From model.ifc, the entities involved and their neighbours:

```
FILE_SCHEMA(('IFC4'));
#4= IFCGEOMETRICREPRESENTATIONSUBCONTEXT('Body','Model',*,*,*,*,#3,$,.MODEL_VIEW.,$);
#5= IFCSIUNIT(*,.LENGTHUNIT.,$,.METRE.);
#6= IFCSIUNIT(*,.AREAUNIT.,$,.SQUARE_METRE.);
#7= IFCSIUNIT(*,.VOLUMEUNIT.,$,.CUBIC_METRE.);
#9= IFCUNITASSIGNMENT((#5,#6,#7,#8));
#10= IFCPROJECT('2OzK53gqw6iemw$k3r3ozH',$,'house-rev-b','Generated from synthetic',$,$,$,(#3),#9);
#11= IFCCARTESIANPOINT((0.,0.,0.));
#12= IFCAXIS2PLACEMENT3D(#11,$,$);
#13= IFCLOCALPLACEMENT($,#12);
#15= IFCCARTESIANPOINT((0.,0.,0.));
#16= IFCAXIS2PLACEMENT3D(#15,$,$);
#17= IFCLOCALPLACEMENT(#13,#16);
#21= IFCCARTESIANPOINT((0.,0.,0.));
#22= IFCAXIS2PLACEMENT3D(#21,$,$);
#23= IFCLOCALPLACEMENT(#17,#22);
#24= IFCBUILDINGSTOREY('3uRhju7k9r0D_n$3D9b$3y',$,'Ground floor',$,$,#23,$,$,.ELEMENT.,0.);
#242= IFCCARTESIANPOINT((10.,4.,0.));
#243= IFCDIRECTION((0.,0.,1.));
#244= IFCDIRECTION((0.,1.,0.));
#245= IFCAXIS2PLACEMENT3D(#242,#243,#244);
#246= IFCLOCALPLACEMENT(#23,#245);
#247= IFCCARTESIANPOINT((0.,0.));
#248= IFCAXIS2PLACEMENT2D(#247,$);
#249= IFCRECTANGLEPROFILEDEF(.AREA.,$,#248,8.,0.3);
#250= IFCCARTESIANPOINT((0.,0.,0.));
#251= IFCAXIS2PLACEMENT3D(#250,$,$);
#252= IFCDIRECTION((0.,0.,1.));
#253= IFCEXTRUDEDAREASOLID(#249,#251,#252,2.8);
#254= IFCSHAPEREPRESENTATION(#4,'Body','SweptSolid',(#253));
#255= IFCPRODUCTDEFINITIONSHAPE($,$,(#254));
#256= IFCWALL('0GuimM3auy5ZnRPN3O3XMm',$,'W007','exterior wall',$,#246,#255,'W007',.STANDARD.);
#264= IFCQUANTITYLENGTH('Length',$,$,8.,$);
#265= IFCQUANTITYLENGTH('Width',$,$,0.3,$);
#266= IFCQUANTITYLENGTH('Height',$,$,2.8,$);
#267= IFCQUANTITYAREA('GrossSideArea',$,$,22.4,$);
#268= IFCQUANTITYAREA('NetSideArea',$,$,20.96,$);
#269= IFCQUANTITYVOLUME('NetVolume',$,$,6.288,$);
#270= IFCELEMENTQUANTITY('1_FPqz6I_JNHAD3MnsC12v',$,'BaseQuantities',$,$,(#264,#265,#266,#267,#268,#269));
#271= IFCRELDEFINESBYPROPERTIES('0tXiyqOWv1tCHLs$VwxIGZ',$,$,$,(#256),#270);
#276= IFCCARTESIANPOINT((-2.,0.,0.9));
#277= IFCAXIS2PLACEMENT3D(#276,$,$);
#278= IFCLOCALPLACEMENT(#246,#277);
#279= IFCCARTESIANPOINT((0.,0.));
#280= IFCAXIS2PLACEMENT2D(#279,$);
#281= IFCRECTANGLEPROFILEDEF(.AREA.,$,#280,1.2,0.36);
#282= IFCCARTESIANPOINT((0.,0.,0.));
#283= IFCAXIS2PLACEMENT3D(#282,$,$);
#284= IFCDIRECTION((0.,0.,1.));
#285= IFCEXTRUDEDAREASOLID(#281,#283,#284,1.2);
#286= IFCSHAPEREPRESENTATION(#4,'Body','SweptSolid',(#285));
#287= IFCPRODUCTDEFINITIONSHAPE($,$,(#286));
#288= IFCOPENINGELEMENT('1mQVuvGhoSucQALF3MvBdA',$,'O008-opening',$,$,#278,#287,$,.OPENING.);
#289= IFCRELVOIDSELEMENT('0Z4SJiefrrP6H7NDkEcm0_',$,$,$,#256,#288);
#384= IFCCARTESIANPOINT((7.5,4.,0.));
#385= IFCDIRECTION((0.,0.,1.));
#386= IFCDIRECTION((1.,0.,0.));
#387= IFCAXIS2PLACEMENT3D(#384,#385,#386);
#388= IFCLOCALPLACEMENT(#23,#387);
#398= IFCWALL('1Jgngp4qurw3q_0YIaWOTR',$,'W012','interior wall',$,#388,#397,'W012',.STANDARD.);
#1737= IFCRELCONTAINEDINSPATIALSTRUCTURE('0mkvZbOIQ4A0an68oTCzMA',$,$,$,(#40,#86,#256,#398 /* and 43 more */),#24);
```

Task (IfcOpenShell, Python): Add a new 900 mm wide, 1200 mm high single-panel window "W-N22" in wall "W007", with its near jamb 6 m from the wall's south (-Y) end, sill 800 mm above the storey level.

```python
import numpy as np
import ifcopenshell
import ifcopenshell.api.feature
import ifcopenshell.api.geometry
import ifcopenshell.api.pset
import ifcopenshell.api.root
import ifcopenshell.api.spatial
import ifcopenshell.geom
import ifcopenshell.util.element
import ifcopenshell.util.placement
import ifcopenshell.util.representation
import ifcopenshell.util.shape
import ifcopenshell.util.unit

model = ifcopenshell.open("model.ifc")
unit_scale = ifcopenshell.util.unit.calculate_unit_scale(model)
area_scale = ifcopenshell.util.unit.calculate_unit_scale(model, "AREAUNIT")
volume_scale = ifcopenshell.util.unit.calculate_unit_scale(model, "VOLUMEUNIT")
settings = ifcopenshell.geom.settings()


def volume(element):
    """Net volume in cubic metres, openings subtracted."""
    shape = ifcopenshell.geom.create_shape(settings, element)
    return ifcopenshell.util.shape.get_volume(shape.geometry)


wall = model.by_guid("0GuimM3auy5ZnRPN3O3XMm")
storey = ifcopenshell.util.element.get_container(wall, ifc_class="IfcBuildingStorey")
context = ifcopenshell.util.representation.get_context(model, "Model", "Body", "MODEL_VIEW")
before = volume(wall)

width, height, from_end, sill = 0.9, 1.2, 6, 0.8  # metres

# The wall runs along its own X axis, and the end named is its -X end.
wall_shape = ifcopenshell.geom.create_shape(settings, wall)
x, y, z = ifcopenshell.util.shape.get_vertices(wall_shape.geometry).T
start = x.min() + from_end
face, thickness = float(y.min()), float(y.max() - y.min())
wall_matrix = ifcopenshell.util.placement.get_local_placement(wall.ObjectPlacement)
level = ifcopenshell.util.placement.get_local_placement(storey.ObjectPlacement)[2, 3]


def in_wall(x, y):
    """Placement at x, y metres in the wall's axes, at sill height."""
    matrix = wall_matrix.copy()
    matrix[:, 3] = wall_matrix @ np.array([x / unit_scale, y / unit_scale, 0.0, 1.0])
    matrix[2, 3] = level + sill / unit_scale
    return matrix


# Opening: a box that overshoots both wall faces by 50 mm.
opening = ifcopenshell.api.root.create_entity(model, ifc_class="IfcOpeningElement", predefined_type="OPENING")
box = ifcopenshell.api.geometry.add_wall_representation(
    model, context=context, length=width, height=height, thickness=thickness + 0.1
)
ifcopenshell.api.geometry.assign_representation(model, product=opening, representation=box)
ifcopenshell.api.geometry.edit_object_placement(model, product=opening, matrix=in_wall(start, face - 0.05), is_si=False)
ifcopenshell.api.feature.add_feature(model, feature=opening, element=wall)

window = ifcopenshell.api.root.create_entity(model, ifc_class="IfcWindow", name="W-N22", predefined_type="WINDOW")
window.OverallWidth, window.OverallHeight = width / unit_scale, height / unit_scale
window.PartitioningType = "SINGLE_PANEL"
body = ifcopenshell.api.geometry.add_window_representation(
    model,
    context=context,
    overall_width=window.OverallWidth,
    overall_height=window.OverallHeight,
    partition_type="SINGLE_PANEL",
)
ifcopenshell.api.geometry.assign_representation(model, product=window, representation=body)
ifcopenshell.api.spatial.assign_container(model, products=[window], relating_structure=storey)
ifcopenshell.api.feature.add_filling(model, opening=opening, element=window)

# Centre the window in the wall's thickness.
ifcopenshell.api.geometry.edit_object_placement(model, product=window, matrix=in_wall(start, face), is_si=False)
window_shape = ifcopenshell.geom.create_shape(settings, window)
depth = ifcopenshell.util.shape.get_vertices(window_shape.geometry)[:, 1]
offset = face + thickness / 2 - (depth.min() + depth.max()) / 2
ifcopenshell.api.geometry.edit_object_placement(model, product=window, matrix=in_wall(start, offset), is_si=False)

after = volume(wall)

# Update the wall's stored quantities.
qto = model.by_id(ifcopenshell.util.element.get_pset(wall, "BaseQuantities", should_inherit=False)["id"])
ifcopenshell.api.pset.edit_qto(model, qto=qto, properties={
    "NetSideArea": after / thickness / area_scale,
    "NetVolume": after / volume_scale,
})

print(f"wall volume {before:.3f} -> {after:.3f} m3")

model.write("model_edited.ifc")
```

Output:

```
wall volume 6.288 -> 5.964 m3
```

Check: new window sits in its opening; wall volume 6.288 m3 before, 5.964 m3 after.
